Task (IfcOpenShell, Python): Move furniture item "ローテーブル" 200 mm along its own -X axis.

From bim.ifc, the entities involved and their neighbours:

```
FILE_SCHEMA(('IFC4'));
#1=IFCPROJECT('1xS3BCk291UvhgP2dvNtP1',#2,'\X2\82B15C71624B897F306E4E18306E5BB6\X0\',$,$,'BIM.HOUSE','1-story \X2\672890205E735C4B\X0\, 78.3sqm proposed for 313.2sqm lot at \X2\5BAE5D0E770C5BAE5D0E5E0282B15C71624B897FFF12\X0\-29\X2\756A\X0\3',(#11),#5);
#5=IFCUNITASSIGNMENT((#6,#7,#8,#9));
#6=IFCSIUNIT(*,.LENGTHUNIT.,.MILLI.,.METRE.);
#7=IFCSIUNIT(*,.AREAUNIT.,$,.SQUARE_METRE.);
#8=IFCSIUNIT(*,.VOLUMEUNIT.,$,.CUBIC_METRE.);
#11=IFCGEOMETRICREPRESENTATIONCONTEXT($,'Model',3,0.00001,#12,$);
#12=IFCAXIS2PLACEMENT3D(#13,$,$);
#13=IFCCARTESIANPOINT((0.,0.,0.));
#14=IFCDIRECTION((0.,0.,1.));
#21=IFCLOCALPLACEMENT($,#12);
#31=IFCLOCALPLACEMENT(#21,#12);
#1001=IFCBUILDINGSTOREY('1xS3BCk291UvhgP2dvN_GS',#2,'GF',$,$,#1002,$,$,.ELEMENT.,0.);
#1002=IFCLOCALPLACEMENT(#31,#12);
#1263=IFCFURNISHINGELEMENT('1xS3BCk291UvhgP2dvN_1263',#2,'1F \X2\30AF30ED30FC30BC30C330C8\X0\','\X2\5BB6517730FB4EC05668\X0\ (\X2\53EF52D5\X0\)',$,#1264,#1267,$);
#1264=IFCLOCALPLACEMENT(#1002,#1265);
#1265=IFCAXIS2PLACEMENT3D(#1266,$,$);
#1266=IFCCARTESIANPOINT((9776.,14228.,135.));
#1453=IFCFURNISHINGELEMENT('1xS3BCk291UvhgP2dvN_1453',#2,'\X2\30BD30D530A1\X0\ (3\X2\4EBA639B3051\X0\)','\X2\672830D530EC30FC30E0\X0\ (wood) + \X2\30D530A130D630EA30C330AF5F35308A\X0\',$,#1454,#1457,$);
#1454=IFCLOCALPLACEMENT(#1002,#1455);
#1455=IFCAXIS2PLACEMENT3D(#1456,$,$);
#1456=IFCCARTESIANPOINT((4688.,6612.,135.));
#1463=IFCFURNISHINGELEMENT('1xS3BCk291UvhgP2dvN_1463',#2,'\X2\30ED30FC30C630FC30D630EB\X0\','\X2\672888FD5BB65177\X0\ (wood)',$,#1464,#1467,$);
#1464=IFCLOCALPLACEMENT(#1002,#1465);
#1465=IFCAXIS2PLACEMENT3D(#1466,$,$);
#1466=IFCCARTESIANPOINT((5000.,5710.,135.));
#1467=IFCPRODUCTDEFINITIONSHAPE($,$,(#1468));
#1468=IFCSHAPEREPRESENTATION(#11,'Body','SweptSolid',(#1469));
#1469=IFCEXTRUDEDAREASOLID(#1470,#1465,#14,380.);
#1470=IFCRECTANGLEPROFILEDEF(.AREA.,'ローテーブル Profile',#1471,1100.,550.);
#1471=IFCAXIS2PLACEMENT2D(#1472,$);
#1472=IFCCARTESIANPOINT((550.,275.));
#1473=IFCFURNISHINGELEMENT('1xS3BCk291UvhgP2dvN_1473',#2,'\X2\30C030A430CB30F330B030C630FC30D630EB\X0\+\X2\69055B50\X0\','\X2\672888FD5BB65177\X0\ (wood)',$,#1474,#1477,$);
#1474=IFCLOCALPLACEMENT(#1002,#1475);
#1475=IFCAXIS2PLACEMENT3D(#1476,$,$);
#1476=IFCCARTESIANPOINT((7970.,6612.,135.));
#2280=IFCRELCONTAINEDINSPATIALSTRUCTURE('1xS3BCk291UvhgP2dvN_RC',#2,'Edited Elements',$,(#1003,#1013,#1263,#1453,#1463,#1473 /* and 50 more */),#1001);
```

```python
import ifcopenshell
import ifcopenshell.api.geometry
import ifcopenshell.util.placement
import ifcopenshell.util.unit

model = ifcopenshell.open("bim.ifc")
unit_scale = ifcopenshell.util.unit.calculate_unit_scale(model)

item = model.by_guid("1xS3BCk291UvhgP2dvN_1463")
matrix = ifcopenshell.util.placement.get_local_placement(item.ObjectPlacement)
matrix[:3, 3] -= matrix[:3, 0] * 0.2 / unit_scale
ifcopenshell.api.geometry.edit_object_placement(model, product=item, matrix=matrix, is_si=False)

print(ifcopenshell.util.placement.get_local_placement(item.ObjectPlacement).round(3) + 0.0)

model.write("bim_v2.ifc")
```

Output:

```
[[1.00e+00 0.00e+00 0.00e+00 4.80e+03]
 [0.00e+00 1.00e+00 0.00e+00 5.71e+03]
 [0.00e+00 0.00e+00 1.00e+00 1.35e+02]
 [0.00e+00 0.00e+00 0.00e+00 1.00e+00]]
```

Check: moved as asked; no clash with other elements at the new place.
